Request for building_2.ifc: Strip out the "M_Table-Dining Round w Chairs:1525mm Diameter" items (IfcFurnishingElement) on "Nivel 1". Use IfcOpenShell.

First a look at what the model holds.

```python
import ifcopenshell
import ifcopenshell.util.element

model = ifcopenshell.open("building_2.ifc")
print(model.schema)
storey = next(s for s in model.by_type("IfcBuildingStorey") if s.Name == "Nivel 1")
furniture = [e for e in ifcopenshell.util.element.get_decomposition(storey) if e.is_a("IfcFurnishingElement")]
seen = {}
for e in furniture:
    element_type = ifcopenshell.util.element.get_type(e)
    name = element_type.Name if element_type not in (None, e) else None
    seen[name] = seen.get(name, 0) + 1
for name, count in sorted(seen.items(), key=str):
    print(count, "x", name)
```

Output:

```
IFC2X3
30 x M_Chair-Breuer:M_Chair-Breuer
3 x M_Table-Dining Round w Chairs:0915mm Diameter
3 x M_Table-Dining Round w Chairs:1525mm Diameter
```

```python
import ifcopenshell
import ifcopenshell.api.root
import ifcopenshell.util.element

model = ifcopenshell.open("building_2.ifc")

storey = next(s for s in model.by_type("IfcBuildingStorey") if s.Name == "Nivel 1")
furniture = [e for e in ifcopenshell.util.element.get_decomposition(storey) if e.is_a("IfcFurnishingElement")]
targets = [e for e in furniture if (t := ifcopenshell.util.element.get_type(e)) not in (None, e) and t.Name == "M_Table-Dining Round w Chairs:1525mm Diameter"]

for e in targets:
    ifcopenshell.api.root.remove_product(model, product=e)
print(len(targets), "removed")

model.write("building_2_edited.ifc")
```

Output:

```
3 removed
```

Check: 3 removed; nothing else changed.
